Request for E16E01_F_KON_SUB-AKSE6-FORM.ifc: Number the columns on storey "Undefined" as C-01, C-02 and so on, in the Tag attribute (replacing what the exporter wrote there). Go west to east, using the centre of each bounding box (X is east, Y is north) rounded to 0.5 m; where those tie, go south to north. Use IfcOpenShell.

First a look at what the model holds.

```python
import ifcopenshell
import ifcopenshell.util.element
import ifcopenshell.util.placement

model = ifcopenshell.open("E16E01_F_KON_SUB-AKSE6-FORM.ifc")
print(model.schema)
storey = next(s for s in model.by_type("IfcBuildingStorey") if s.Name == "Undefined")
columns = [e for e in ifcopenshell.util.element.get_decomposition(storey) if e.is_a("IfcColumn")]
for e in sorted(columns, key=lambda e: e.id()):
    origin = ifcopenshell.util.placement.get_local_placement(e.ObjectPlacement)[:3, 3]
    print(e.id(), e.Tag, e.Name, origin.round(2) + 0.0, sep=" | ")
```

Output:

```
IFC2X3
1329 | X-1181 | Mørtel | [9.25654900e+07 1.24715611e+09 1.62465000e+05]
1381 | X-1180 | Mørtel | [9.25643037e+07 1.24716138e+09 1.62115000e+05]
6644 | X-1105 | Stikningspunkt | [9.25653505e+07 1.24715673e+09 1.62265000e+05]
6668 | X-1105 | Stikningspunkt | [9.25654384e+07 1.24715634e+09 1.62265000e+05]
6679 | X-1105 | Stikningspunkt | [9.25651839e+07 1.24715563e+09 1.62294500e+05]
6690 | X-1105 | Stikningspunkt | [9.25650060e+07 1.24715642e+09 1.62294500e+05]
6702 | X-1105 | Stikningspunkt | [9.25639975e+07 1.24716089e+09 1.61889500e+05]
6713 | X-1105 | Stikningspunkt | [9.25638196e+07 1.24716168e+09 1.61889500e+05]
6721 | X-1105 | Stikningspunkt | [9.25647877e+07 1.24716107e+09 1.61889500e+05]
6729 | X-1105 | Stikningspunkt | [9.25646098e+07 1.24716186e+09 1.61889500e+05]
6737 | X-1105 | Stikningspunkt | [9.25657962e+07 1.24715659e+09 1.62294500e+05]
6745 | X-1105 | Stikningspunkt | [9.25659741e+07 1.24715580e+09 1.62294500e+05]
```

```python
import ifcopenshell
import ifcopenshell.geom
import ifcopenshell.util.element
import ifcopenshell.util.shape

model = ifcopenshell.open("E16E01_F_KON_SUB-AKSE6-FORM.ifc")
settings = ifcopenshell.geom.settings()
settings.set("use-world-coords", True)


def centre(element):
    shape = ifcopenshell.geom.create_shape(settings, element)
    return ifcopenshell.util.shape.get_bbox_centroid(shape.geometry)


storey = next(s for s in model.by_type("IfcBuildingStorey") if s.Name == "Undefined")
columns = [e for e in ifcopenshell.util.element.get_decomposition(storey) if e.is_a("IfcColumn")]

# Insertion points can sit at a corner or the storey origin, so sort by the geometry (in metres).
centres = {e: centre(e) for e in columns}
columns.sort(key=lambda e: (round(centres[e][0] / 0.5), centres[e][1]))

for i, e in enumerate(columns, start=1):
    number = f"C-{i:02d}"
    e.Tag = number
    print(e.id(), number)

model.write("E16E01_F_KON_SUB-AKSE6-FORM_rev.ifc")
```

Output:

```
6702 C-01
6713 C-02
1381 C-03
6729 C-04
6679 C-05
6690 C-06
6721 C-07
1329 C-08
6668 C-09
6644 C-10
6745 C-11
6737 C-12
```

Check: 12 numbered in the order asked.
